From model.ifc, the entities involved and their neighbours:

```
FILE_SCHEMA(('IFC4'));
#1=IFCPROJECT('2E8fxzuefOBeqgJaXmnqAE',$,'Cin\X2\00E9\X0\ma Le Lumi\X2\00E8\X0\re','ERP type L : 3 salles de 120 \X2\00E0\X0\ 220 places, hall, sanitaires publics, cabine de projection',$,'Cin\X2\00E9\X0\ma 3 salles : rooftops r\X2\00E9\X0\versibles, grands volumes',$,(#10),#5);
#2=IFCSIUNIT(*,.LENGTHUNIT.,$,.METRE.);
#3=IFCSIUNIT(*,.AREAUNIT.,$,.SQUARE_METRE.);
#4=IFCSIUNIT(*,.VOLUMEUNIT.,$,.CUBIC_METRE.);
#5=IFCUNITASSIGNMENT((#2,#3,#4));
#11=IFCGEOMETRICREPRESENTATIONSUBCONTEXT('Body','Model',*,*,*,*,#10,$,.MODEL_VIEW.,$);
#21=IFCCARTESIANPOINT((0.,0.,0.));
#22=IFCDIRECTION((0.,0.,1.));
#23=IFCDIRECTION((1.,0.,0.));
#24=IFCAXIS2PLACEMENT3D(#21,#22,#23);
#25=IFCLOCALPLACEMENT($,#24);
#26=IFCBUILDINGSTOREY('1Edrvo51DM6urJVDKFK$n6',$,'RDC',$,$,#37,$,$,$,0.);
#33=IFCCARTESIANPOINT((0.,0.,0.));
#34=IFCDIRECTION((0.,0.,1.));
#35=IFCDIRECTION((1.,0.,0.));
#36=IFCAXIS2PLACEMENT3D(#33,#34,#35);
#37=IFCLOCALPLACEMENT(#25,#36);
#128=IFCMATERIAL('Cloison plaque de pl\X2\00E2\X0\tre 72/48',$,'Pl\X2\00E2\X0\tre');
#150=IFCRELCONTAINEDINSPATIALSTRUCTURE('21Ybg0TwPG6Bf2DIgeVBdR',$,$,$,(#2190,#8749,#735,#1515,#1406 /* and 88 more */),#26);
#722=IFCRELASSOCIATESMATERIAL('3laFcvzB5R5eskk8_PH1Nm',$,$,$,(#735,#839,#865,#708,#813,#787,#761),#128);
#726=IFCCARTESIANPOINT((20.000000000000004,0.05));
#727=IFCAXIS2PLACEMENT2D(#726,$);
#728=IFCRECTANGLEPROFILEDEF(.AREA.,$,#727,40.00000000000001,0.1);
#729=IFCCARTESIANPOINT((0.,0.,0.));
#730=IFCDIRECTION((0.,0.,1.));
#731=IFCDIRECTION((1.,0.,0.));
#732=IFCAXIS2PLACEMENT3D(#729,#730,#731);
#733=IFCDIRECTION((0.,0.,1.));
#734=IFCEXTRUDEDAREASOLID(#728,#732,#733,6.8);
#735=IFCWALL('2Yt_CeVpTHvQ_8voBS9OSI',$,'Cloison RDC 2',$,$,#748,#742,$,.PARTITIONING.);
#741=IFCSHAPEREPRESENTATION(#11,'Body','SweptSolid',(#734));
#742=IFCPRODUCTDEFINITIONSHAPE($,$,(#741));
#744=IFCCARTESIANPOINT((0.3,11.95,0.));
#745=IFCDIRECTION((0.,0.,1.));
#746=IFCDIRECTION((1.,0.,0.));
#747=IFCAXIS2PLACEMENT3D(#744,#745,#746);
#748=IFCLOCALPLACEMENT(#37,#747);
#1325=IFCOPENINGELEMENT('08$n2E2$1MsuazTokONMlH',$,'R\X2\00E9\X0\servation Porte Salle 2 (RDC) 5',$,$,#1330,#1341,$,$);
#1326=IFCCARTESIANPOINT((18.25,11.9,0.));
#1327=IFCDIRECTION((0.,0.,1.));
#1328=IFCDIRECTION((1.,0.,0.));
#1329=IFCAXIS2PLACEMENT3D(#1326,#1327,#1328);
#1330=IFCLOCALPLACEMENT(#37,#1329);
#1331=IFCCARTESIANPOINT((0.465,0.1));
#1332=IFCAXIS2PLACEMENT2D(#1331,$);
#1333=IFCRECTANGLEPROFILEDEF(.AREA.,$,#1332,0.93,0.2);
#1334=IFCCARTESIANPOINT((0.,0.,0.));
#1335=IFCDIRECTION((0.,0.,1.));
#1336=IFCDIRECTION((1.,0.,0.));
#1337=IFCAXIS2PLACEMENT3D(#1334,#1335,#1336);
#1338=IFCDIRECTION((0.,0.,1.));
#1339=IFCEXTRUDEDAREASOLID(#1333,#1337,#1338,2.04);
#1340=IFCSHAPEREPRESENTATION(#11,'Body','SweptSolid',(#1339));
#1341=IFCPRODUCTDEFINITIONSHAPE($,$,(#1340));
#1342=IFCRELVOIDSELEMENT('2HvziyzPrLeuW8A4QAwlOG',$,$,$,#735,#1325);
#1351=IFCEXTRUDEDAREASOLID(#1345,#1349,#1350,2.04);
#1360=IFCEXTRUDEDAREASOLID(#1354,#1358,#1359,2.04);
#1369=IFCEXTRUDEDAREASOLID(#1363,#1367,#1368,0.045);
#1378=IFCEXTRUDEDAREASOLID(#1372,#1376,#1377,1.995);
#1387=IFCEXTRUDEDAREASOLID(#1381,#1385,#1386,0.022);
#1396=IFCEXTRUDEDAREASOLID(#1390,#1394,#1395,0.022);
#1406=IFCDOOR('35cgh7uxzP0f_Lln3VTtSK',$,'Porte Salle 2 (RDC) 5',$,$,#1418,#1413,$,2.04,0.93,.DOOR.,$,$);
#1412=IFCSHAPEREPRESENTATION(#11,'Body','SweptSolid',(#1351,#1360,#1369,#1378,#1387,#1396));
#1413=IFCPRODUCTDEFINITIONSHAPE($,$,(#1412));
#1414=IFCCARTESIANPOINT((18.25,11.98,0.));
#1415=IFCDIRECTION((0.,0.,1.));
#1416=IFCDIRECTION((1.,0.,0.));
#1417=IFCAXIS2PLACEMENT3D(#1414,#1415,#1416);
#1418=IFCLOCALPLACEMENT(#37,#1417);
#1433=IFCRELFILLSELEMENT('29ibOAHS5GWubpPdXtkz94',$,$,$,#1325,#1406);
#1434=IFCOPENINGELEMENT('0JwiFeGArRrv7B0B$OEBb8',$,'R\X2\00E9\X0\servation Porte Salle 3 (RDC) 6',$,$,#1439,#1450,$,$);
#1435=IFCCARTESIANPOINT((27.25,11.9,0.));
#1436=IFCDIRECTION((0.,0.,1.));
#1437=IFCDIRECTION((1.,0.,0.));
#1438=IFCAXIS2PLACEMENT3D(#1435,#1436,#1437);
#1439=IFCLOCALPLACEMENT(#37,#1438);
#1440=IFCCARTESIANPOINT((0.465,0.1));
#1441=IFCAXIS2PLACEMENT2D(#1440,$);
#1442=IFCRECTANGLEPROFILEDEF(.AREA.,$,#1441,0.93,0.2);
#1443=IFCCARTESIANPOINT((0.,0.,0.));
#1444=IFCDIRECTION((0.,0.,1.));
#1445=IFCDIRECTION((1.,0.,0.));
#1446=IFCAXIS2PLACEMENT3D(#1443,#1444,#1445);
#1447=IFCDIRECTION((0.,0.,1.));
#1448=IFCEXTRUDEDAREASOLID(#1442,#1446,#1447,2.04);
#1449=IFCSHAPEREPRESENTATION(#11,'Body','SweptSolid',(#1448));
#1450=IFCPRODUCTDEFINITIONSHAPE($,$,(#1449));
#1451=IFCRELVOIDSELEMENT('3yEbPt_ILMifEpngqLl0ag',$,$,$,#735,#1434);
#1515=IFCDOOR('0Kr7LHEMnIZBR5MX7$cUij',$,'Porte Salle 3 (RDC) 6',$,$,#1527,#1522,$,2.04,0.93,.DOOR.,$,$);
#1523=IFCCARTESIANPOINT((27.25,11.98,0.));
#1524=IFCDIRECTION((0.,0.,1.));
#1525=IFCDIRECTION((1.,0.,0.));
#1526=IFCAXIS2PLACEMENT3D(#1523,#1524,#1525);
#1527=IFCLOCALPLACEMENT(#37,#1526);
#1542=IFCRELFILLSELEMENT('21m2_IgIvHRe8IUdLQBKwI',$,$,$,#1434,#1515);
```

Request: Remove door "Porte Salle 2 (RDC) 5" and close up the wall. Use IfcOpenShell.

```python
import ifcopenshell
import ifcopenshell.api.feature
import ifcopenshell.api.root
import ifcopenshell.geom
import ifcopenshell.util.shape

model = ifcopenshell.open("model.ifc")
settings = ifcopenshell.geom.settings()


def volume(element):
    """Net volume in cubic metres, openings subtracted."""
    shape = ifcopenshell.geom.create_shape(settings, element)
    return ifcopenshell.util.shape.get_volume(shape.geometry)


door = model.by_guid("35cgh7uxzP0f_Lln3VTtSK")
opening = door.FillsVoids[0].RelatingOpeningElement
wall = opening.VoidsElements[0].RelatingBuildingElement
before = volume(wall)

ifcopenshell.api.root.remove_product(model, product=door)
ifcopenshell.api.feature.remove_feature(model, feature=opening)

after = volume(wall)

print(f"wall volume {before:.3f} -> {after:.3f} m3")

model.write("model_edited.ifc")
```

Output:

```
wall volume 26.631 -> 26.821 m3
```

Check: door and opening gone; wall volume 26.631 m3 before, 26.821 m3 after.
